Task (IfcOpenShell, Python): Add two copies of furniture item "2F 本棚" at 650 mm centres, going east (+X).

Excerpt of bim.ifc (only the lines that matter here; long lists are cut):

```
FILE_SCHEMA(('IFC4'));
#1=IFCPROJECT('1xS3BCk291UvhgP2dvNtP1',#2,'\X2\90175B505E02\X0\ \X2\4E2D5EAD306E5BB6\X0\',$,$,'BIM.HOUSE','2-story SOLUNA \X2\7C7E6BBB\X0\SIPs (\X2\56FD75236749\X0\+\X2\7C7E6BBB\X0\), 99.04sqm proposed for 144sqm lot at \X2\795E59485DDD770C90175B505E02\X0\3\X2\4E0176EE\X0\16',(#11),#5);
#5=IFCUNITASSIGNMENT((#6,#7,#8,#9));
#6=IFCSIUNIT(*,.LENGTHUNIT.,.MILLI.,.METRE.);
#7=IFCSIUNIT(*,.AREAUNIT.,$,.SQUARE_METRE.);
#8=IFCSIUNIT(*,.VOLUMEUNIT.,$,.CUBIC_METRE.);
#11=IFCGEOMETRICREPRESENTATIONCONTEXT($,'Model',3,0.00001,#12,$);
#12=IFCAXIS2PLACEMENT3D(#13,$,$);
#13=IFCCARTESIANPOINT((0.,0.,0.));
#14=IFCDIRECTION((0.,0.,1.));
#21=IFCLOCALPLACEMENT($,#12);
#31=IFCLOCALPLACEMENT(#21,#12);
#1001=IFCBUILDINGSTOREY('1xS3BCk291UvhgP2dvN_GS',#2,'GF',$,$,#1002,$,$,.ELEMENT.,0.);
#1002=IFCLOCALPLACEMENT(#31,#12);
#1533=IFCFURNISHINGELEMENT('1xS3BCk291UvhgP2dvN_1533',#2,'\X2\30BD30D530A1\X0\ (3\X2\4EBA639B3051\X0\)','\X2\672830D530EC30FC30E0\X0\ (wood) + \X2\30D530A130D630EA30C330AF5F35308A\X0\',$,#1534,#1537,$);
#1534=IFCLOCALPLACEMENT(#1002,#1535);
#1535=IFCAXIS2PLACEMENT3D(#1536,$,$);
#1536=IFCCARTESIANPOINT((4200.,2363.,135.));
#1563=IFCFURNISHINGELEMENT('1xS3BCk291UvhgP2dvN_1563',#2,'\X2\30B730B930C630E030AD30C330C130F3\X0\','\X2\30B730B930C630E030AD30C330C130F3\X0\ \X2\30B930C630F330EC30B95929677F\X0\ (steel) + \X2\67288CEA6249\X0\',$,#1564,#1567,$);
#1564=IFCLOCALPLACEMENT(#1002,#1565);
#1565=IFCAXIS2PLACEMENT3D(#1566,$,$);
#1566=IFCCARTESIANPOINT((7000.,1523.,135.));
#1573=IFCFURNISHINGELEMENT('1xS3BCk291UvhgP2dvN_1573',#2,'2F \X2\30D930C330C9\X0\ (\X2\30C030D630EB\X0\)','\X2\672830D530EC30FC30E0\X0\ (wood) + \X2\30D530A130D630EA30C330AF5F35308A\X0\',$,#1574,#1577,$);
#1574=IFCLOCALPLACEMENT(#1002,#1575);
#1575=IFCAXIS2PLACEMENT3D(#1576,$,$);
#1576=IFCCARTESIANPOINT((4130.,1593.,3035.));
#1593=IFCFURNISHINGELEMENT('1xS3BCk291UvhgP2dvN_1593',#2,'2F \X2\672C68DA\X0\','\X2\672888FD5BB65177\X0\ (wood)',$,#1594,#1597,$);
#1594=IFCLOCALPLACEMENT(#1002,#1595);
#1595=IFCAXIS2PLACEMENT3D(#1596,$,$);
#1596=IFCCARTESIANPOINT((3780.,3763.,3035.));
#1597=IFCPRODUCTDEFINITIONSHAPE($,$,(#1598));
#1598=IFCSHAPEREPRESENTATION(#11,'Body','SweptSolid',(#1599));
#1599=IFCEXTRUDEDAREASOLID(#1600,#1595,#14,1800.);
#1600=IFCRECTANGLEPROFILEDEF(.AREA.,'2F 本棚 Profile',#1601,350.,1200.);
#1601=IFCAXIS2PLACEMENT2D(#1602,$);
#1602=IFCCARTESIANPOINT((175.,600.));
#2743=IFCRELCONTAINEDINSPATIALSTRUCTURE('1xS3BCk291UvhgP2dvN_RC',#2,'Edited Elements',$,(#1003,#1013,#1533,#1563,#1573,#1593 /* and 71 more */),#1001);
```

```python
import numpy as np
import ifcopenshell
import ifcopenshell.api.geometry
import ifcopenshell.api.root
import ifcopenshell.util.element
import ifcopenshell.util.placement

model = ifcopenshell.open("bim.ifc")


def reuse_history(source, copy):
    """copy_class also copies each property set's owner history, people and application; keep the originals."""
    for rel in copy.IsDefinedBy:
        if rel.is_a("IfcRelDefinesByProperties") and (history := rel.RelatingPropertyDefinition.OwnerHistory):
            rel.RelatingPropertyDefinition.OwnerHistory = source.OwnerHistory
            ifcopenshell.util.element.remove_deep2(model, history)


source = model.by_guid("1xS3BCk291UvhgP2dvN_1593")
base = ifcopenshell.util.placement.get_local_placement(source.ObjectPlacement)
step = np.array([1.0, 0.0, 0.0]) * 650.0

for i in range(1, 3):
    copy = ifcopenshell.api.root.copy_class(model, product=source)
    copy.Representation = ifcopenshell.util.element.copy_deep(
        model, source.Representation, exclude=["IfcGeometricRepresentationContext", "IfcRepresentationMap"]
    )
    reuse_history(source, copy)
    matrix = base.copy()
    matrix[:3, 3] += i * step
    print("added at", matrix[:3, 3].round(3) + 0.0)
    ifcopenshell.api.geometry.edit_object_placement(model, product=copy, matrix=matrix, is_si=False)

model.write("bim_edited.ifc")
```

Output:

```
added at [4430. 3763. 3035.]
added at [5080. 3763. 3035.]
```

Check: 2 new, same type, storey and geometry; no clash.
